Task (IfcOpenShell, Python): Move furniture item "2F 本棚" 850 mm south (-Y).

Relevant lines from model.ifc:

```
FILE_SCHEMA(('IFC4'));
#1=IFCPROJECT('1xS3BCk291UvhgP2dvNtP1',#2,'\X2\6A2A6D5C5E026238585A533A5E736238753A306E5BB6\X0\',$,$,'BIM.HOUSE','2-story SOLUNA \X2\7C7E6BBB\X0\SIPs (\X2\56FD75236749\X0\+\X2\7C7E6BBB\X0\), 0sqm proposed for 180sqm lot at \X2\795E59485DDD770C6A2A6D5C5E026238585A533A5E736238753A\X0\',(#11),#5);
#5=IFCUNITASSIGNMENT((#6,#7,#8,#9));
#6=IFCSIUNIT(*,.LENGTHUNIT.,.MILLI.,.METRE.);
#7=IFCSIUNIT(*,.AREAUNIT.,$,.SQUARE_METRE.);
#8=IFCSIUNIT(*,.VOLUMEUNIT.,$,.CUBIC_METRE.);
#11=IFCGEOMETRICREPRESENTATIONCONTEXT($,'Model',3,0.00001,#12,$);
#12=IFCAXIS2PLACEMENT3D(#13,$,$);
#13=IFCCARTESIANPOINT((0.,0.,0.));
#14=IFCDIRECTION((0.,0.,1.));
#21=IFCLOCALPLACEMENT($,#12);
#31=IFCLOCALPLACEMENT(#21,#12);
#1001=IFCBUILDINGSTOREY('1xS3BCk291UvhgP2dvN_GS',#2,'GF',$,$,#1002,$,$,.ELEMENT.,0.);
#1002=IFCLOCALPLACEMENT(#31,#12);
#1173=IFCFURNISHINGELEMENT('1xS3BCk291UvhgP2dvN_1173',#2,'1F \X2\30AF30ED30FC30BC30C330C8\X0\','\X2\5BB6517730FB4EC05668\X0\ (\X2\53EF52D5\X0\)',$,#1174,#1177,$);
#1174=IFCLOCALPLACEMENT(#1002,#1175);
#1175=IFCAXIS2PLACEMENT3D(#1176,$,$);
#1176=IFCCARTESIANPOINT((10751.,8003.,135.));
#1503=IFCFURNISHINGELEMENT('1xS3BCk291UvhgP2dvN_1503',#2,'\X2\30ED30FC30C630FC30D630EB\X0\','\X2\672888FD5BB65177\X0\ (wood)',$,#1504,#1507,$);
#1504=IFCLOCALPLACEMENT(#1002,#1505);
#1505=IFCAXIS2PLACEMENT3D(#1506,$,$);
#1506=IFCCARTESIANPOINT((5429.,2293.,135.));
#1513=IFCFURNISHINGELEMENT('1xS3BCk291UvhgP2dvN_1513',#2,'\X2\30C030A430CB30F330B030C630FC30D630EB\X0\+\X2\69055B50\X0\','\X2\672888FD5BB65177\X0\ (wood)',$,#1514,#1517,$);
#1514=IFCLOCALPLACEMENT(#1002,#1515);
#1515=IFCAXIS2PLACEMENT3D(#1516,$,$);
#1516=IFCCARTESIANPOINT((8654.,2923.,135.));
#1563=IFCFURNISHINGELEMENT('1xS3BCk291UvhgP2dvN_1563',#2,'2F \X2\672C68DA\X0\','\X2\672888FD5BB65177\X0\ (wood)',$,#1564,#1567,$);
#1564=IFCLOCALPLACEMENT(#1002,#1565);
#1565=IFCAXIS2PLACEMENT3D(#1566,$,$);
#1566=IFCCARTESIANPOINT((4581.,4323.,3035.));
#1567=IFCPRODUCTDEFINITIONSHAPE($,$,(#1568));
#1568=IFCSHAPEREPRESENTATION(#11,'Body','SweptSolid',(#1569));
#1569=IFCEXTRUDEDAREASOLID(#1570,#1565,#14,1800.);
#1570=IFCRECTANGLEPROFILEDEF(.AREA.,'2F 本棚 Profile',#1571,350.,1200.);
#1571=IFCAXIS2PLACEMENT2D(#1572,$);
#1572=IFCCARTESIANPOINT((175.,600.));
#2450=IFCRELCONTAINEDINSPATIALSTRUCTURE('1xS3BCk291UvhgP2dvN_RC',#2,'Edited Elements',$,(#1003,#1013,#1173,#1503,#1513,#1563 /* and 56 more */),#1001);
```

```python
import ifcopenshell
import ifcopenshell.api.geometry
import ifcopenshell.util.placement
import ifcopenshell.util.unit

model = ifcopenshell.open("model.ifc")
unit_scale = ifcopenshell.util.unit.calculate_unit_scale(model)

item = model.by_guid("1xS3BCk291UvhgP2dvN_1563")
matrix = ifcopenshell.util.placement.get_local_placement(item.ObjectPlacement)
matrix[1, 3] -= 0.85 / unit_scale
ifcopenshell.api.geometry.edit_object_placement(model, product=item, matrix=matrix, is_si=False)

print(ifcopenshell.util.placement.get_local_placement(item.ObjectPlacement).round(3) + 0.0)

model.write("model_rev.ifc")
```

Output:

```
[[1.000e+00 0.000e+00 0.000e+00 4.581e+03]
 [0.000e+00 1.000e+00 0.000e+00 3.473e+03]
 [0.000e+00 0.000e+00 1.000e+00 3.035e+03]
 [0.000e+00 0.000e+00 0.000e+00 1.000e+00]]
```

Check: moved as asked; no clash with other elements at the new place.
